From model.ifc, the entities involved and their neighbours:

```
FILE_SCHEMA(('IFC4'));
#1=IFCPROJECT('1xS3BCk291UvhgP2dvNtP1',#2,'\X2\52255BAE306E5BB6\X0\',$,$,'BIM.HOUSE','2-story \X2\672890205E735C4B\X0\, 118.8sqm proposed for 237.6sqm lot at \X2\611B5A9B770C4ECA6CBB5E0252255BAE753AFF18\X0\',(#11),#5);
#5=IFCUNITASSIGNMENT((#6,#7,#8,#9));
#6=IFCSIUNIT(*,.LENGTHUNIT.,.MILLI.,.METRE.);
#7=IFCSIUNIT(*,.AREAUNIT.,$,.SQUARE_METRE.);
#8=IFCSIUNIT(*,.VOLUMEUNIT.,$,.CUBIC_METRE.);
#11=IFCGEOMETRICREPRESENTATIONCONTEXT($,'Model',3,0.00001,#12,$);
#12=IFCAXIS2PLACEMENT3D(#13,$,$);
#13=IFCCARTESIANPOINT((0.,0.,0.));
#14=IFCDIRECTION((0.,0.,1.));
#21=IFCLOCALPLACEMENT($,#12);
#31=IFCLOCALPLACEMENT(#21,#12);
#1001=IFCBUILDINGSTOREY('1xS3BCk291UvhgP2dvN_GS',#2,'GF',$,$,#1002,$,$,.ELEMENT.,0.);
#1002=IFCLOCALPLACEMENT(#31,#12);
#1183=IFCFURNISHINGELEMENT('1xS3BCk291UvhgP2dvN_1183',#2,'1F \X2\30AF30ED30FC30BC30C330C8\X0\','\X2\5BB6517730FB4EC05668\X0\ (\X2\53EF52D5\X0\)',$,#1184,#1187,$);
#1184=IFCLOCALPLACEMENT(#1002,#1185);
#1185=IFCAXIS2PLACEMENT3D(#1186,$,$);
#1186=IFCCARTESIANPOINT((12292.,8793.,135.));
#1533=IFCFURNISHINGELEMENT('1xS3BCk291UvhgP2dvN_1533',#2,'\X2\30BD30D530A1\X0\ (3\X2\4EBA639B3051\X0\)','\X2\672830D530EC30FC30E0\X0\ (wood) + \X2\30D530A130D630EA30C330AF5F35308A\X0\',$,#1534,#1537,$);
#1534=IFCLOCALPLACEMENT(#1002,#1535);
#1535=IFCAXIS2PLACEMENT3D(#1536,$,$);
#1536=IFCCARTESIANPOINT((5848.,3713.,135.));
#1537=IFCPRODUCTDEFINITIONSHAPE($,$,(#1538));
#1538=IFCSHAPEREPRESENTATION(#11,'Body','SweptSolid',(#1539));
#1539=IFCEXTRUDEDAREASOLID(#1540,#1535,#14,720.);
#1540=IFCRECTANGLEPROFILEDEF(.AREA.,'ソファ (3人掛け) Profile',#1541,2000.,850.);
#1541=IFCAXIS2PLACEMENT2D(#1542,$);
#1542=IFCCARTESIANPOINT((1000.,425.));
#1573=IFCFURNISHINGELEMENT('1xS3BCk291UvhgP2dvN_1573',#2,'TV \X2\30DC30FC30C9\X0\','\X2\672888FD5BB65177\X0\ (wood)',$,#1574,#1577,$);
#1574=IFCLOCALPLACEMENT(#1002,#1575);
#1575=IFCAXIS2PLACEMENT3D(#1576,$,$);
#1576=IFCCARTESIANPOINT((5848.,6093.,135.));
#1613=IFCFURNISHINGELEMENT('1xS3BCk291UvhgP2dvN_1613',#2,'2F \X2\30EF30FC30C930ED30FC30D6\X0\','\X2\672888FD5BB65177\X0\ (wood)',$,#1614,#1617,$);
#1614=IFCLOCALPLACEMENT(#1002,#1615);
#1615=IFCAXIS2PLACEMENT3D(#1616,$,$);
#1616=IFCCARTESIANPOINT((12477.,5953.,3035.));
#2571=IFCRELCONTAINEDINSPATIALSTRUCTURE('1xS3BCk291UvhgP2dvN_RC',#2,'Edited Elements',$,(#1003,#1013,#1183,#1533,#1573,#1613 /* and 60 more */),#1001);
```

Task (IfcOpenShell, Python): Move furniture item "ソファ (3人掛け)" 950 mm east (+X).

```python
import ifcopenshell
import ifcopenshell.api.geometry
import ifcopenshell.util.placement
import ifcopenshell.util.unit

model = ifcopenshell.open("model.ifc")
unit_scale = ifcopenshell.util.unit.calculate_unit_scale(model)

item = model.by_guid("1xS3BCk291UvhgP2dvN_1533")
matrix = ifcopenshell.util.placement.get_local_placement(item.ObjectPlacement)
matrix[0, 3] += 0.95 / unit_scale
ifcopenshell.api.geometry.edit_object_placement(model, product=item, matrix=matrix, is_si=False)

print(ifcopenshell.util.placement.get_local_placement(item.ObjectPlacement).round(3) + 0.0)

model.write("model_updated.ifc")
```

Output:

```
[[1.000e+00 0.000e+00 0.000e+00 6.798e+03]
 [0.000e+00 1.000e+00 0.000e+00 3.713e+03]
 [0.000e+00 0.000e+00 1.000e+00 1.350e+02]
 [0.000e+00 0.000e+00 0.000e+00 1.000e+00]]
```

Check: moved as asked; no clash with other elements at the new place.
